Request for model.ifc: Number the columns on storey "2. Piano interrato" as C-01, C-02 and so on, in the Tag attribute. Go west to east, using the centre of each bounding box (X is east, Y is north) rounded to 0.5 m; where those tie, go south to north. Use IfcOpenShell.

First a look at what the model holds.

```python
import ifcopenshell
import ifcopenshell.util.element
import ifcopenshell.util.placement

model = ifcopenshell.open("model.ifc")
print(model.schema)
storey = next(s for s in model.by_type("IfcBuildingStorey") if s.Name == "2. Piano interrato")
columns = [e for e in ifcopenshell.util.element.get_decomposition(storey) if e.is_a("IfcColumn")]
for e in sorted(columns, key=lambda e: e.id()):
    origin = ifcopenshell.util.placement.get_local_placement(e.ObjectPlacement)[:3, 3]
    print(e.id(), e.Tag, e.Name, origin.round(2) + 0.0, sep=" | ")
```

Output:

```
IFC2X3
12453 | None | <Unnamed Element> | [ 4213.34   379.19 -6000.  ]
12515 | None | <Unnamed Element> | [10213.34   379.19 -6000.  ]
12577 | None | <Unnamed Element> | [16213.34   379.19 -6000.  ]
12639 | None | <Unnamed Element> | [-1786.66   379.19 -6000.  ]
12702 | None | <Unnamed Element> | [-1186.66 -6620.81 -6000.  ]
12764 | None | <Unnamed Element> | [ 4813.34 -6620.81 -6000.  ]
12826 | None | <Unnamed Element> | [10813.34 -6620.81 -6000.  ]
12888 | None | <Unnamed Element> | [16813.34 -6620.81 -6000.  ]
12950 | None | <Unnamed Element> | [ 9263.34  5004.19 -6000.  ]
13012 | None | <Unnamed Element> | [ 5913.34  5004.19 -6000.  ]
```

```python
import ifcopenshell
import ifcopenshell.geom
import ifcopenshell.util.element
import ifcopenshell.util.shape

model = ifcopenshell.open("model.ifc")
settings = ifcopenshell.geom.settings()
settings.set("use-world-coords", True)


def centre(element):
    shape = ifcopenshell.geom.create_shape(settings, element)
    return ifcopenshell.util.shape.get_bbox_centroid(shape.geometry)


storey = next(s for s in model.by_type("IfcBuildingStorey") if s.Name == "2. Piano interrato")
columns = [e for e in ifcopenshell.util.element.get_decomposition(storey) if e.is_a("IfcColumn")]

# Insertion points can sit at a corner or the storey origin, so sort by the geometry (in metres).
centres = {e: centre(e) for e in columns}
columns.sort(key=lambda e: (round(centres[e][0] / 0.5), centres[e][1]))

for i, e in enumerate(columns, start=1):
    number = f"C-{i:02d}"
    e.Tag = number
    print(e.id(), number)

model.write("model_updated.ifc")
```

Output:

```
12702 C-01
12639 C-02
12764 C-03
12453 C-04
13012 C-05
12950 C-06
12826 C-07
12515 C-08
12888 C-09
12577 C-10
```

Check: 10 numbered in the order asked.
